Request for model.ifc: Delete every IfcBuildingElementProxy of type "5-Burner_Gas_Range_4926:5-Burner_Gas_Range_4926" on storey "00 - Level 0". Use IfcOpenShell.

First a look at what the model holds.

```python
import ifcopenshell
import ifcopenshell.util.element

model = ifcopenshell.open("model.ifc")
print(model.schema)
storey = next(s for s in model.by_type("IfcBuildingStorey") if s.Name == "00 - Level 0")
proxies = [e for e in ifcopenshell.util.element.get_decomposition(storey) if e.is_a("IfcBuildingElementProxy")]
seen = {}
for e in proxies:
    element_type = ifcopenshell.util.element.get_type(e)
    name = element_type.Name if element_type not in (None, e) else None
    seen[name] = seen.get(name, 0) + 1
for name, count in sorted(seen.items(), key=str):
    print(count, "x", name)
```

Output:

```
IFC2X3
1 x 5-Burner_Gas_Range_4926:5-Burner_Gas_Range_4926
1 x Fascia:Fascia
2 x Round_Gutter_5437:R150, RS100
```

```python
import ifcopenshell
import ifcopenshell.api.root
import ifcopenshell.util.element

model = ifcopenshell.open("model.ifc")

storey = next(s for s in model.by_type("IfcBuildingStorey") if s.Name == "00 - Level 0")
proxies = [e for e in ifcopenshell.util.element.get_decomposition(storey) if e.is_a("IfcBuildingElementProxy")]
targets = [e for e in proxies if (t := ifcopenshell.util.element.get_type(e)) not in (None, e) and t.Name == "5-Burner_Gas_Range_4926:5-Burner_Gas_Range_4926"]

for e in targets:
    ifcopenshell.api.root.remove_product(model, product=e)
print(len(targets), "removed")

model.write("model_edited.ifc")
```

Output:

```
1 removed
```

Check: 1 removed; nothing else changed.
